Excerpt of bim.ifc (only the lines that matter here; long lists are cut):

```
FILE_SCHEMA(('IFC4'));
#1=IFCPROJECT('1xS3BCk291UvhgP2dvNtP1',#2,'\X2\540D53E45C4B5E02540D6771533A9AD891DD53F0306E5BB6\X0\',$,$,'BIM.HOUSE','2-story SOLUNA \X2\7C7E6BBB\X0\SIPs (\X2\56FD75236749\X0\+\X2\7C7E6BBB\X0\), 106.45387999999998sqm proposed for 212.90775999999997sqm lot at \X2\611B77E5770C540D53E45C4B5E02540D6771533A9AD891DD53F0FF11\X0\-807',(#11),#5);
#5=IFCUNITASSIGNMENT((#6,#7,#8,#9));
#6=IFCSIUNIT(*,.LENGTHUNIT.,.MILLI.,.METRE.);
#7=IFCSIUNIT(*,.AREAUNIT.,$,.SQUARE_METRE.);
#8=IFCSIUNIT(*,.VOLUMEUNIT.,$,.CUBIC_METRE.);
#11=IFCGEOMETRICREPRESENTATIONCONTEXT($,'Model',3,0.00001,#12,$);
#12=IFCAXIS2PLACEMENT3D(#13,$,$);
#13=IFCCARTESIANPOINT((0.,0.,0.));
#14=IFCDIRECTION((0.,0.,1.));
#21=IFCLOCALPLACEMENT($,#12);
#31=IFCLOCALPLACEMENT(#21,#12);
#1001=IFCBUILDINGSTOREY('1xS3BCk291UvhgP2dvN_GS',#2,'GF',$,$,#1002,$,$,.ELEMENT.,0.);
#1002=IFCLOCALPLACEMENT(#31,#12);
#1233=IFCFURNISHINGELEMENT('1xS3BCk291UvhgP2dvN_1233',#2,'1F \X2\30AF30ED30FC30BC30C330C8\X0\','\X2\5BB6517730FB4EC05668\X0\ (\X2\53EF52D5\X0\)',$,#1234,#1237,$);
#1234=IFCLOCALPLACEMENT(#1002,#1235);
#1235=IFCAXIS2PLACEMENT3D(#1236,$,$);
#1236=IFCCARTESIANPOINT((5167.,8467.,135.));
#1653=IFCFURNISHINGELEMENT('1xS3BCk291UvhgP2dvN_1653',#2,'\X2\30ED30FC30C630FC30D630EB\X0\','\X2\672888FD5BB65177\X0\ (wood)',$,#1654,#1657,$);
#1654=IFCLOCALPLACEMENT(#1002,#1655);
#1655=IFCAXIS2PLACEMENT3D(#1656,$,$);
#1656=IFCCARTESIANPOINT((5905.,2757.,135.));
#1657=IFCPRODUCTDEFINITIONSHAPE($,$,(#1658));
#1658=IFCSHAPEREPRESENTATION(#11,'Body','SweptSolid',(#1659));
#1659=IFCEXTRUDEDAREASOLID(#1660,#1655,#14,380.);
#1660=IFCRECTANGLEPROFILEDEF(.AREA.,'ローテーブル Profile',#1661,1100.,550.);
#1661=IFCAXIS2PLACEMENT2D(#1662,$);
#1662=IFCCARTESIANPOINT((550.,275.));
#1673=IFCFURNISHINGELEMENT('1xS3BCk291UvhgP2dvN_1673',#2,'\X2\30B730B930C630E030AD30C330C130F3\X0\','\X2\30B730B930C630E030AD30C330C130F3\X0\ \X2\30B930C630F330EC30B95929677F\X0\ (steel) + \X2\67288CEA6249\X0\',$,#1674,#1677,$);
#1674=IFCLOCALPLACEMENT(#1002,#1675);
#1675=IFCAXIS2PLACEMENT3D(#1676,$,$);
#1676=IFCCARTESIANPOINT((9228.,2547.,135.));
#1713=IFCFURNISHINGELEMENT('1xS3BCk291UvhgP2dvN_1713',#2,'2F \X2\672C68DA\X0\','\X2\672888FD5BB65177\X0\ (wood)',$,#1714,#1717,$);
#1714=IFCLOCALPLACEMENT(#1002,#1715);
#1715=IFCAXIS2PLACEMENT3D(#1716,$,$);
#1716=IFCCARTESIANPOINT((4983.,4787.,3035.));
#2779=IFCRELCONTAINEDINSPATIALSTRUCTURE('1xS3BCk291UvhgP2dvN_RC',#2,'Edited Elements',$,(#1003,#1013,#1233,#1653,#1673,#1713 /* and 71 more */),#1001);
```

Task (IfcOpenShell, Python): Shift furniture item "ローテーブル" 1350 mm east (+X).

```python
import ifcopenshell
import ifcopenshell.api.geometry
import ifcopenshell.util.placement

model = ifcopenshell.open("bim.ifc")

item = model.by_guid("1xS3BCk291UvhgP2dvN_1653")
matrix = ifcopenshell.util.placement.get_local_placement(item.ObjectPlacement)
matrix[0, 3] += 1350.0
ifcopenshell.api.geometry.edit_object_placement(model, product=item, matrix=matrix, is_si=False)

print(ifcopenshell.util.placement.get_local_placement(item.ObjectPlacement).round(3) + 0.0)

model.write("bim-out.ifc")
```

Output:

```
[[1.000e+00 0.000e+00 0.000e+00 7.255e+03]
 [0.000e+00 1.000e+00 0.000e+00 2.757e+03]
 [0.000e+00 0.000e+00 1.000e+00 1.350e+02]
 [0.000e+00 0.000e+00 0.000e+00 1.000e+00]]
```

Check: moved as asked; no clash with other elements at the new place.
